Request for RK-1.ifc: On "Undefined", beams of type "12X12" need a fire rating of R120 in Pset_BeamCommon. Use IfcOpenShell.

First a look at what the model holds.

```python
import ifcopenshell
import ifcopenshell.util.element

model = ifcopenshell.open("RK-1.ifc")
print(model.schema)
storey = next(s for s in model.by_type("IfcBuildingStorey") if s.Name == "Undefined")
beams = [e for e in ifcopenshell.util.element.get_decomposition(storey) if e.is_a("IfcBeam")]
seen = {}
for e in beams:
    element_type = ifcopenshell.util.element.get_type(e)
    key = (element_type.Name if element_type != e and element_type else None, ifcopenshell.util.element.get_pset(e, "Pset_BeamCommon", "FireRating"))
    seen[key] = seen.get(key, 0) + 1
for (name, value), count in sorted(seen.items(), key=str):
    print(count, "x", name, "|", value)
```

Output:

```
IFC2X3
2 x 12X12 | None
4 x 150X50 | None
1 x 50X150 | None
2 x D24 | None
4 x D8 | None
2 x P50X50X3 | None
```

```python
import ifcopenshell
import ifcopenshell.api.pset
import ifcopenshell.util.element

model = ifcopenshell.open("RK-1.ifc")

storey = next(s for s in model.by_type("IfcBuildingStorey") if s.Name == "Undefined")
beams = [e for e in ifcopenshell.util.element.get_decomposition(storey) if e.is_a("IfcBeam")]

count = 0
for e in beams:
    element_type = ifcopenshell.util.element.get_type(e)
    if element_type in (None, e) or element_type.Name != "12X12":
        continue
    found = ifcopenshell.util.element.get_pset(e, "Pset_BeamCommon", should_inherit=False)
    if found:
        pset = model.by_id(found["id"])
        if len(ifcopenshell.util.element.get_elements_by_pset(pset)) > 1:
            pset = ifcopenshell.api.pset.unshare_pset(model, products=[e], pset=pset)[0]
    else:
        pset = ifcopenshell.api.pset.add_pset(model, product=e, name="Pset_BeamCommon")
    ifcopenshell.api.pset.edit_pset(model, pset=pset, properties={"FireRating": "R120"})
    count += 1

print(count, "beams updated")

model.write("RK-1_v2.ifc")
```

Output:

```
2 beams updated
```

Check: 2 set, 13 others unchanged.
